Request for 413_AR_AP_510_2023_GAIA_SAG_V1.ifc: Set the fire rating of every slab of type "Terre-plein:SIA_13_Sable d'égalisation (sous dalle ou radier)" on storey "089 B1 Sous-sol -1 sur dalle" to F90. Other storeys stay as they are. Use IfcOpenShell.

First a look at what the model holds.

```python
import ifcopenshell
import ifcopenshell.util.element

model = ifcopenshell.open("413_AR_AP_510_2023_GAIA_SAG_V1.ifc")
print(model.schema)
storey = next(s for s in model.by_type("IfcBuildingStorey") if s.Name == "089 B1 Sous-sol -1 sur dalle")
slabs = [e for e in ifcopenshell.util.element.get_decomposition(storey) if e.is_a("IfcSlab")]
seen = {}
for e in slabs:
    element_type = ifcopenshell.util.element.get_type(e)
    key = (element_type.Name if element_type != e and element_type else None, ifcopenshell.util.element.get_pset(e, "Pset_SlabCommon", "FireRating"))
    seen[key] = seen.get(key, 0) + 1
for (name, value), count in sorted(seen.items(), key=str):
    print(count, "x", name, "|", value)
```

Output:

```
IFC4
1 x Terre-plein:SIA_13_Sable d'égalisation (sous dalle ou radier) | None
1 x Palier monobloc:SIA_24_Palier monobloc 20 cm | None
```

```python
import ifcopenshell
import ifcopenshell.api.pset
import ifcopenshell.util.element

model = ifcopenshell.open("413_AR_AP_510_2023_GAIA_SAG_V1.ifc")

storey = next(s for s in model.by_type("IfcBuildingStorey") if s.Name == "089 B1 Sous-sol -1 sur dalle")
slabs = [e for e in ifcopenshell.util.element.get_decomposition(storey) if e.is_a("IfcSlab")]

count = 0
for e in slabs:
    element_type = ifcopenshell.util.element.get_type(e)
    if element_type in (None, e) or element_type.Name != "Terre-plein:SIA_13_Sable d'égalisation (sous dalle ou radier)":
        continue
    # add_pset returns the element's existing set when there is one.
    pset = ifcopenshell.api.pset.add_pset(model, product=e, name="Pset_SlabCommon")
    ifcopenshell.api.pset.edit_pset(model, pset=pset, properties={"FireRating": "F90"})
    count += 1

print(count, "slabs updated")

model.write("413_AR_AP_510_2023_GAIA_SAG_V1_v2.ifc")
```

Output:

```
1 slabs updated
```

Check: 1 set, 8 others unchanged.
